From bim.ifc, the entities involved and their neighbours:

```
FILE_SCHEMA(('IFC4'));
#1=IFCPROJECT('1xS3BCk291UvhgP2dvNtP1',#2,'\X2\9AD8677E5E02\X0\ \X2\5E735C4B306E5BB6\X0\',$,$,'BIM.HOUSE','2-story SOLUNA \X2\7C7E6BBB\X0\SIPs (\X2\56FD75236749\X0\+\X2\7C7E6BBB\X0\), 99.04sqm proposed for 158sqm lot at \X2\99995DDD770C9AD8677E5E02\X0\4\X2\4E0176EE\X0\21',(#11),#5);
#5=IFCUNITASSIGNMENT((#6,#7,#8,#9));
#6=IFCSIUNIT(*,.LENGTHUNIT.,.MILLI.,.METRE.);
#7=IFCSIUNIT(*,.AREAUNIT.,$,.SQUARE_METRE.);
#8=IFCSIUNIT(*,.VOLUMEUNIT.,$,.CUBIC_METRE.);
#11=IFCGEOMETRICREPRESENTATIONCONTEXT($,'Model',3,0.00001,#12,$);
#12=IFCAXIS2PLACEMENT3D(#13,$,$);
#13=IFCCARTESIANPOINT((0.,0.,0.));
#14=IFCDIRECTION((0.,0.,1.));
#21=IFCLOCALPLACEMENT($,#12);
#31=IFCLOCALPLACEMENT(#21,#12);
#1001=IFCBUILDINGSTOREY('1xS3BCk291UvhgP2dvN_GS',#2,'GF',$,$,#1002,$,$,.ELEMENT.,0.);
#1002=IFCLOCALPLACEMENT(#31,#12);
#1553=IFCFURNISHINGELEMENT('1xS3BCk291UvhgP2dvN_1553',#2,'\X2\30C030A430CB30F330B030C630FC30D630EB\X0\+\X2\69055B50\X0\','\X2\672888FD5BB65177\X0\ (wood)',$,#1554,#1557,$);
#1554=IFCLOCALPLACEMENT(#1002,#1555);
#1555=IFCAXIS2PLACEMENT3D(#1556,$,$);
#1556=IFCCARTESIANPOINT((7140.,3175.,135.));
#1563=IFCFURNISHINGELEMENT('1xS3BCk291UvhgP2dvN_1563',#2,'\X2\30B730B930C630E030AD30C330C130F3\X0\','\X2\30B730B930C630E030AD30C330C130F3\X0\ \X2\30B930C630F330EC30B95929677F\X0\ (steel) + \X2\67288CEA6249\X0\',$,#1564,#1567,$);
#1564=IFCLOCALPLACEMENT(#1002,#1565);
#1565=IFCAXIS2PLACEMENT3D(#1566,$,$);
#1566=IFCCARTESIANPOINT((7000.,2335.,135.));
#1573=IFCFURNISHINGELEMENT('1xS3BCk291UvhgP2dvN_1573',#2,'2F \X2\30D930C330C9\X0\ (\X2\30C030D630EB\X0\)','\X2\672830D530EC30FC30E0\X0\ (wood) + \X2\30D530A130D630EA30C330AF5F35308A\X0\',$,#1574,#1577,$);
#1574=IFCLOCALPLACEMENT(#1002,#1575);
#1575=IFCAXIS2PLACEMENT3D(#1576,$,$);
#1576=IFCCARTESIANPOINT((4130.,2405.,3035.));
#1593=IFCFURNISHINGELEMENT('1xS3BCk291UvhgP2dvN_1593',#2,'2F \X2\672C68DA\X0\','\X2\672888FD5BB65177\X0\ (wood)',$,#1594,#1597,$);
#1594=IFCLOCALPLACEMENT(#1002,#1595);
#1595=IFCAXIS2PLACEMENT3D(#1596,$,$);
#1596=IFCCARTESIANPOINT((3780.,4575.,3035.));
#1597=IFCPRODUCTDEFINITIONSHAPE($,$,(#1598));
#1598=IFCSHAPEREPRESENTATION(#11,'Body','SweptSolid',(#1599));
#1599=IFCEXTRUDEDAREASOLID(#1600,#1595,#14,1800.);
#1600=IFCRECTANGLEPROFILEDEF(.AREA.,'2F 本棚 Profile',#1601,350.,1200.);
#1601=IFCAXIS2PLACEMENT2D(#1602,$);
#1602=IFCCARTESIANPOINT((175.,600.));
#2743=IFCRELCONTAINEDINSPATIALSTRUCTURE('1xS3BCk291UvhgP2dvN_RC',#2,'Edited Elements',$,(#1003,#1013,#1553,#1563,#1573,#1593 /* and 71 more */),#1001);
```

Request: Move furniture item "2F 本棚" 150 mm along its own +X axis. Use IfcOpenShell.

```python
import ifcopenshell
import ifcopenshell.api.geometry
import ifcopenshell.util.placement
import ifcopenshell.util.unit

model = ifcopenshell.open("bim.ifc")
unit_scale = ifcopenshell.util.unit.calculate_unit_scale(model)

item = model.by_guid("1xS3BCk291UvhgP2dvN_1593")
matrix = ifcopenshell.util.placement.get_local_placement(item.ObjectPlacement)
matrix[:3, 3] += matrix[:3, 0] * 0.15 / unit_scale
ifcopenshell.api.geometry.edit_object_placement(model, product=item, matrix=matrix, is_si=False)

print(ifcopenshell.util.placement.get_local_placement(item.ObjectPlacement).round(3) + 0.0)

model.write("bim_v2.ifc")
```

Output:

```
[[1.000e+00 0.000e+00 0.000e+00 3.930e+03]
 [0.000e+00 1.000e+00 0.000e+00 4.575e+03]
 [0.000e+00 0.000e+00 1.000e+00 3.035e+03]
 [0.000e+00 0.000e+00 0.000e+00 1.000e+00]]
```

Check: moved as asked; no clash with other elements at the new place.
